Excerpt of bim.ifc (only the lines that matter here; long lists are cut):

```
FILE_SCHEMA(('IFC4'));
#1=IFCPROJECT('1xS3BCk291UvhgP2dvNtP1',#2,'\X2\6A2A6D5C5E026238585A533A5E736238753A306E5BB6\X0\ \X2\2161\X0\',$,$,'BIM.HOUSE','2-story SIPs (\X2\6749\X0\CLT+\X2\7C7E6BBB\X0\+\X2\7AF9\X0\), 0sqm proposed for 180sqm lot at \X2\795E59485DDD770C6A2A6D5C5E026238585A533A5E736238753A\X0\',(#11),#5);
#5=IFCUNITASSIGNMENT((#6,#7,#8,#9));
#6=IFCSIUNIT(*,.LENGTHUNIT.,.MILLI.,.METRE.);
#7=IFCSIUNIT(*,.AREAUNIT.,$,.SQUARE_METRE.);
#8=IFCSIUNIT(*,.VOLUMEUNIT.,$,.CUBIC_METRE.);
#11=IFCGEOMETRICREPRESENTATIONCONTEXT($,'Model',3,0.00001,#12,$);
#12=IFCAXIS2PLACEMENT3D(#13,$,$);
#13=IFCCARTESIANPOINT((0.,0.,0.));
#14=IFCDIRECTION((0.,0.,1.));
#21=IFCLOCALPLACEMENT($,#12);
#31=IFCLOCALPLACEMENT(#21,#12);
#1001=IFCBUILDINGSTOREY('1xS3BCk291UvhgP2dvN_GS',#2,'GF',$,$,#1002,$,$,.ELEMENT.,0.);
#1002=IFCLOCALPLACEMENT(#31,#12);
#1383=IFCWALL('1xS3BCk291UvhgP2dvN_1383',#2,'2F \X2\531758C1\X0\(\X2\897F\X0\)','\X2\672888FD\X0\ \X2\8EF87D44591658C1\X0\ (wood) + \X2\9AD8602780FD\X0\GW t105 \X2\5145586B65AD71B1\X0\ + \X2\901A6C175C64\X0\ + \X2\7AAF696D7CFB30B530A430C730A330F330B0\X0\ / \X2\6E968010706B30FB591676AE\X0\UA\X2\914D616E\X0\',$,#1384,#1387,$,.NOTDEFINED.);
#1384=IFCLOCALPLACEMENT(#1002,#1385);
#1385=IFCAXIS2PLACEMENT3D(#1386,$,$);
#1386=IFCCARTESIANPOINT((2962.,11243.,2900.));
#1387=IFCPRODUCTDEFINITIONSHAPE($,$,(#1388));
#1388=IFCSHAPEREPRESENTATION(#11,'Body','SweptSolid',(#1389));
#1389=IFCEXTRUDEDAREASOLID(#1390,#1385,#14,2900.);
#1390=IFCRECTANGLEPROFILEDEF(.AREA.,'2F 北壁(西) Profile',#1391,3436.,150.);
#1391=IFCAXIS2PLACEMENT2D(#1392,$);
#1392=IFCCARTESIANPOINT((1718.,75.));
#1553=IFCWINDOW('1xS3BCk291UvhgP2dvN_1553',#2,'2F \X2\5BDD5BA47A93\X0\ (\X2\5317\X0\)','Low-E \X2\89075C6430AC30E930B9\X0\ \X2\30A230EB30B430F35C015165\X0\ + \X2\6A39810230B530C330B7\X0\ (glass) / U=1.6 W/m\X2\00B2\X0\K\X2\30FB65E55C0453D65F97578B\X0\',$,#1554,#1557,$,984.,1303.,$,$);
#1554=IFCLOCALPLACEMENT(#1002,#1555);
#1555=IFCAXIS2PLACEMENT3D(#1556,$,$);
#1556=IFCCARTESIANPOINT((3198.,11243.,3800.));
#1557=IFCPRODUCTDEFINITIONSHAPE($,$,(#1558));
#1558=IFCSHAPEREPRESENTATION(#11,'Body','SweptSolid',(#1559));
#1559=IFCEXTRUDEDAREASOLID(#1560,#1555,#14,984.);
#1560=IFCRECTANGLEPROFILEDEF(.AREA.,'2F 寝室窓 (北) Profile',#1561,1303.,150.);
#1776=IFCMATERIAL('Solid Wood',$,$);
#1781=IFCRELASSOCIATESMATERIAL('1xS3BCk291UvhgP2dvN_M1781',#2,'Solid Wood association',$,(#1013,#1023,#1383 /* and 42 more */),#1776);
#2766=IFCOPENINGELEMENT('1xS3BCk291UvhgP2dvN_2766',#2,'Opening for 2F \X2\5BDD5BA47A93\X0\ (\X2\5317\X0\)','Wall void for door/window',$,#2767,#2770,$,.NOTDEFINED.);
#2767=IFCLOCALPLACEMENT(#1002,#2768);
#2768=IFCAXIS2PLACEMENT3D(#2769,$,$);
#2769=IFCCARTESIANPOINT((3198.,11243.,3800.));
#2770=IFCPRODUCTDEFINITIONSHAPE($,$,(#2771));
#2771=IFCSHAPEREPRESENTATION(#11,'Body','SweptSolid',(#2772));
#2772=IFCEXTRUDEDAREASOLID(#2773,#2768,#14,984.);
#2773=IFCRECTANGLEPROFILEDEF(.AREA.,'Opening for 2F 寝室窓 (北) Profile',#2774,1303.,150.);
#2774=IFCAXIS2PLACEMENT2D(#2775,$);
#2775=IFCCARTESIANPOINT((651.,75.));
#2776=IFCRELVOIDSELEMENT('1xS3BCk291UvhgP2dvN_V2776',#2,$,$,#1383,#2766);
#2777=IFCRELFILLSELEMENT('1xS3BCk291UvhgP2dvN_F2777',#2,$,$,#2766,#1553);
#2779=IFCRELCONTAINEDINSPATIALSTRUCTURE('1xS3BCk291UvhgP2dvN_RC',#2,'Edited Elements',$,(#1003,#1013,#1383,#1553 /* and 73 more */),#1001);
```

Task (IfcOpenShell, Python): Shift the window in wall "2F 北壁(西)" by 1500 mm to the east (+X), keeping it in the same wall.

```python
import ifcopenshell
import ifcopenshell.api.geometry
import ifcopenshell.util.placement
import ifcopenshell.util.unit

model = ifcopenshell.open("bim.ifc")
unit_scale = ifcopenshell.util.unit.calculate_unit_scale(model)

window = model.by_guid("1xS3BCk291UvhgP2dvN_1553")
opening = window.FillsVoids[0].RelatingOpeningElement
wall = opening.VoidsElements[0].RelatingBuildingElement

wall_matrix = ifcopenshell.util.placement.get_local_placement(wall.ObjectPlacement)
shift = wall_matrix[:3, 0] * 1.5 / unit_scale
before = ifcopenshell.util.placement.get_local_placement(window.ObjectPlacement)[:3, 3].copy()

# The window is not placed relative to its opening, so move both.
for product in (opening, window):
    matrix = ifcopenshell.util.placement.get_local_placement(product.ObjectPlacement)
    matrix[:3, 3] += shift
    ifcopenshell.api.geometry.edit_object_placement(model, product=product, matrix=matrix, is_si=False)

after = ifcopenshell.util.placement.get_local_placement(window.ObjectPlacement)[:3, 3]
print("window moved by", (after - before).round(3) + 0.0)

model.write("bim_updated.ifc")
```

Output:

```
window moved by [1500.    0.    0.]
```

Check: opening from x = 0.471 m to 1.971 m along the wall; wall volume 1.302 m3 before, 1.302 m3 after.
